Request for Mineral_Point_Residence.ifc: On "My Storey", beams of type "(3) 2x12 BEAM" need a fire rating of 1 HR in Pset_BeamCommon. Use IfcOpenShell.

First a look at what the model holds.

```python
import ifcopenshell
import ifcopenshell.util.element

model = ifcopenshell.open("Mineral_Point_Residence.ifc")
print(model.schema)
storey = next(s for s in model.by_type("IfcBuildingStorey") if s.Name == "My Storey")
beams = [e for e in ifcopenshell.util.element.get_decomposition(storey) if e.is_a("IfcBeam")]
seen = {}
for e in beams:
    element_type = ifcopenshell.util.element.get_type(e)
    key = (element_type.Name if element_type != e and element_type else None, ifcopenshell.util.element.get_pset(e, "Pset_BeamCommon", "FireRating"))
    seen[key] = seen.get(key, 0) + 1
for (name, value), count in sorted(seen.items(), key=str):
    print(count, "x", name, "|", value)
```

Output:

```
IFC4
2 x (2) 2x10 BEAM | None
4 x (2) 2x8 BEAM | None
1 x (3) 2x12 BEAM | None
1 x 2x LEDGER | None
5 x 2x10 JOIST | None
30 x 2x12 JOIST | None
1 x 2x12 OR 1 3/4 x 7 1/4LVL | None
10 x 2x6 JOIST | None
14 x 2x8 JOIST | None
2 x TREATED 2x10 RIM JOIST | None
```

```python
import ifcopenshell
import ifcopenshell.api.pset
import ifcopenshell.util.element

model = ifcopenshell.open("Mineral_Point_Residence.ifc")

storey = next(s for s in model.by_type("IfcBuildingStorey") if s.Name == "My Storey")
beams = [e for e in ifcopenshell.util.element.get_decomposition(storey) if e.is_a("IfcBeam")]

count = 0
for e in beams:
    element_type = ifcopenshell.util.element.get_type(e)
    if element_type in (None, e) or element_type.Name != "(3) 2x12 BEAM":
        continue
    # add_pset returns the element's existing set when there is one.
    pset = ifcopenshell.api.pset.add_pset(model, product=e, name="Pset_BeamCommon")
    ifcopenshell.api.pset.edit_pset(model, pset=pset, properties={"FireRating": "1 HR"})
    count += 1

print(count, "beams updated")

model.write("Mineral_Point_Residence_edited.ifc")
```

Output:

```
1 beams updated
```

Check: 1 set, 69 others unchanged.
